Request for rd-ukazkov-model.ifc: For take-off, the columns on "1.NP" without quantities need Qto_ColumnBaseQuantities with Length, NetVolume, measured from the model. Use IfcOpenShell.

First a look at what the model holds.

```python
import ifcopenshell
import ifcopenshell.util.element
import ifcopenshell.util.unit

model = ifcopenshell.open("rd-ukazkov-model.ifc")
print(model.schema)
for unit_type in ("LENGTHUNIT", "AREAUNIT", "VOLUMEUNIT"):
    print(unit_type, ifcopenshell.util.unit.calculate_unit_scale(model, unit_type))
storey = next(s for s in model.by_type("IfcBuildingStorey") if s.Name == "1.NP")
columns = [e for e in ifcopenshell.util.element.get_decomposition(storey) if e.is_a("IfcColumn")]
for e in sorted(columns, key=lambda e: e.id()):
    print(e.id(), e.is_a(), e.Name, list(ifcopenshell.util.element.get_psets(e, qtos_only=True)), sep=" | ")
```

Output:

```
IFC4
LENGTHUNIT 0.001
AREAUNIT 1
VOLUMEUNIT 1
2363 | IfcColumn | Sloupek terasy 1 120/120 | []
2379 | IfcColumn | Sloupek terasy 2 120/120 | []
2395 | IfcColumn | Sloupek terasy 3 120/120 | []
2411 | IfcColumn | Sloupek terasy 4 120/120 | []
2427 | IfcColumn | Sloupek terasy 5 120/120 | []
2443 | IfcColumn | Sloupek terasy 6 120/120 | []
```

```python
import ifcopenshell
import ifcopenshell.api.pset
import ifcopenshell.geom
import ifcopenshell.util.element
import ifcopenshell.util.shape
import ifcopenshell.util.unit

model = ifcopenshell.open("rd-ukazkov-model.ifc")
unit_scale = ifcopenshell.util.unit.calculate_unit_scale(model)
volume_scale = ifcopenshell.util.unit.calculate_unit_scale(model, "VOLUMEUNIT")
settings = ifcopenshell.geom.settings()

storey = next(s for s in model.by_type("IfcBuildingStorey") if s.Name == "1.NP")
columns = [e for e in ifcopenshell.util.element.get_decomposition(storey) if e.is_a("IfcColumn")]

for e in sorted(columns, key=lambda e: e.id()):
    if ifcopenshell.util.element.get_psets(e, qtos_only=True, should_inherit=False):
        continue
    # Geometry comes back in metres, in the element's own axes.
    shape = ifcopenshell.geom.create_shape(settings, e)
    values = {
        "Length": ifcopenshell.util.shape.get_z(shape.geometry) / unit_scale,
        "NetVolume": ifcopenshell.util.shape.get_volume(shape.geometry) / volume_scale,
    }
    qto = ifcopenshell.api.pset.add_qto(model, product=e, name="Qto_ColumnBaseQuantities")
    ifcopenshell.api.pset.edit_qto(model, qto=qto, properties=values)
    print(e.id(), {k: round(v, 3) for k, v in values.items()})

model.write("rd-ukazkov-model-out.ifc")
```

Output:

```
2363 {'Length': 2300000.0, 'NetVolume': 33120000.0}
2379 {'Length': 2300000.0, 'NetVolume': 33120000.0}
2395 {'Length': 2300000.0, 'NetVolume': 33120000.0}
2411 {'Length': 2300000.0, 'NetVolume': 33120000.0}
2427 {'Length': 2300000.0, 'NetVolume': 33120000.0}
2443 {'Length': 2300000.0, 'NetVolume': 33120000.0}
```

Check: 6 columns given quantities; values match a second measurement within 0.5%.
